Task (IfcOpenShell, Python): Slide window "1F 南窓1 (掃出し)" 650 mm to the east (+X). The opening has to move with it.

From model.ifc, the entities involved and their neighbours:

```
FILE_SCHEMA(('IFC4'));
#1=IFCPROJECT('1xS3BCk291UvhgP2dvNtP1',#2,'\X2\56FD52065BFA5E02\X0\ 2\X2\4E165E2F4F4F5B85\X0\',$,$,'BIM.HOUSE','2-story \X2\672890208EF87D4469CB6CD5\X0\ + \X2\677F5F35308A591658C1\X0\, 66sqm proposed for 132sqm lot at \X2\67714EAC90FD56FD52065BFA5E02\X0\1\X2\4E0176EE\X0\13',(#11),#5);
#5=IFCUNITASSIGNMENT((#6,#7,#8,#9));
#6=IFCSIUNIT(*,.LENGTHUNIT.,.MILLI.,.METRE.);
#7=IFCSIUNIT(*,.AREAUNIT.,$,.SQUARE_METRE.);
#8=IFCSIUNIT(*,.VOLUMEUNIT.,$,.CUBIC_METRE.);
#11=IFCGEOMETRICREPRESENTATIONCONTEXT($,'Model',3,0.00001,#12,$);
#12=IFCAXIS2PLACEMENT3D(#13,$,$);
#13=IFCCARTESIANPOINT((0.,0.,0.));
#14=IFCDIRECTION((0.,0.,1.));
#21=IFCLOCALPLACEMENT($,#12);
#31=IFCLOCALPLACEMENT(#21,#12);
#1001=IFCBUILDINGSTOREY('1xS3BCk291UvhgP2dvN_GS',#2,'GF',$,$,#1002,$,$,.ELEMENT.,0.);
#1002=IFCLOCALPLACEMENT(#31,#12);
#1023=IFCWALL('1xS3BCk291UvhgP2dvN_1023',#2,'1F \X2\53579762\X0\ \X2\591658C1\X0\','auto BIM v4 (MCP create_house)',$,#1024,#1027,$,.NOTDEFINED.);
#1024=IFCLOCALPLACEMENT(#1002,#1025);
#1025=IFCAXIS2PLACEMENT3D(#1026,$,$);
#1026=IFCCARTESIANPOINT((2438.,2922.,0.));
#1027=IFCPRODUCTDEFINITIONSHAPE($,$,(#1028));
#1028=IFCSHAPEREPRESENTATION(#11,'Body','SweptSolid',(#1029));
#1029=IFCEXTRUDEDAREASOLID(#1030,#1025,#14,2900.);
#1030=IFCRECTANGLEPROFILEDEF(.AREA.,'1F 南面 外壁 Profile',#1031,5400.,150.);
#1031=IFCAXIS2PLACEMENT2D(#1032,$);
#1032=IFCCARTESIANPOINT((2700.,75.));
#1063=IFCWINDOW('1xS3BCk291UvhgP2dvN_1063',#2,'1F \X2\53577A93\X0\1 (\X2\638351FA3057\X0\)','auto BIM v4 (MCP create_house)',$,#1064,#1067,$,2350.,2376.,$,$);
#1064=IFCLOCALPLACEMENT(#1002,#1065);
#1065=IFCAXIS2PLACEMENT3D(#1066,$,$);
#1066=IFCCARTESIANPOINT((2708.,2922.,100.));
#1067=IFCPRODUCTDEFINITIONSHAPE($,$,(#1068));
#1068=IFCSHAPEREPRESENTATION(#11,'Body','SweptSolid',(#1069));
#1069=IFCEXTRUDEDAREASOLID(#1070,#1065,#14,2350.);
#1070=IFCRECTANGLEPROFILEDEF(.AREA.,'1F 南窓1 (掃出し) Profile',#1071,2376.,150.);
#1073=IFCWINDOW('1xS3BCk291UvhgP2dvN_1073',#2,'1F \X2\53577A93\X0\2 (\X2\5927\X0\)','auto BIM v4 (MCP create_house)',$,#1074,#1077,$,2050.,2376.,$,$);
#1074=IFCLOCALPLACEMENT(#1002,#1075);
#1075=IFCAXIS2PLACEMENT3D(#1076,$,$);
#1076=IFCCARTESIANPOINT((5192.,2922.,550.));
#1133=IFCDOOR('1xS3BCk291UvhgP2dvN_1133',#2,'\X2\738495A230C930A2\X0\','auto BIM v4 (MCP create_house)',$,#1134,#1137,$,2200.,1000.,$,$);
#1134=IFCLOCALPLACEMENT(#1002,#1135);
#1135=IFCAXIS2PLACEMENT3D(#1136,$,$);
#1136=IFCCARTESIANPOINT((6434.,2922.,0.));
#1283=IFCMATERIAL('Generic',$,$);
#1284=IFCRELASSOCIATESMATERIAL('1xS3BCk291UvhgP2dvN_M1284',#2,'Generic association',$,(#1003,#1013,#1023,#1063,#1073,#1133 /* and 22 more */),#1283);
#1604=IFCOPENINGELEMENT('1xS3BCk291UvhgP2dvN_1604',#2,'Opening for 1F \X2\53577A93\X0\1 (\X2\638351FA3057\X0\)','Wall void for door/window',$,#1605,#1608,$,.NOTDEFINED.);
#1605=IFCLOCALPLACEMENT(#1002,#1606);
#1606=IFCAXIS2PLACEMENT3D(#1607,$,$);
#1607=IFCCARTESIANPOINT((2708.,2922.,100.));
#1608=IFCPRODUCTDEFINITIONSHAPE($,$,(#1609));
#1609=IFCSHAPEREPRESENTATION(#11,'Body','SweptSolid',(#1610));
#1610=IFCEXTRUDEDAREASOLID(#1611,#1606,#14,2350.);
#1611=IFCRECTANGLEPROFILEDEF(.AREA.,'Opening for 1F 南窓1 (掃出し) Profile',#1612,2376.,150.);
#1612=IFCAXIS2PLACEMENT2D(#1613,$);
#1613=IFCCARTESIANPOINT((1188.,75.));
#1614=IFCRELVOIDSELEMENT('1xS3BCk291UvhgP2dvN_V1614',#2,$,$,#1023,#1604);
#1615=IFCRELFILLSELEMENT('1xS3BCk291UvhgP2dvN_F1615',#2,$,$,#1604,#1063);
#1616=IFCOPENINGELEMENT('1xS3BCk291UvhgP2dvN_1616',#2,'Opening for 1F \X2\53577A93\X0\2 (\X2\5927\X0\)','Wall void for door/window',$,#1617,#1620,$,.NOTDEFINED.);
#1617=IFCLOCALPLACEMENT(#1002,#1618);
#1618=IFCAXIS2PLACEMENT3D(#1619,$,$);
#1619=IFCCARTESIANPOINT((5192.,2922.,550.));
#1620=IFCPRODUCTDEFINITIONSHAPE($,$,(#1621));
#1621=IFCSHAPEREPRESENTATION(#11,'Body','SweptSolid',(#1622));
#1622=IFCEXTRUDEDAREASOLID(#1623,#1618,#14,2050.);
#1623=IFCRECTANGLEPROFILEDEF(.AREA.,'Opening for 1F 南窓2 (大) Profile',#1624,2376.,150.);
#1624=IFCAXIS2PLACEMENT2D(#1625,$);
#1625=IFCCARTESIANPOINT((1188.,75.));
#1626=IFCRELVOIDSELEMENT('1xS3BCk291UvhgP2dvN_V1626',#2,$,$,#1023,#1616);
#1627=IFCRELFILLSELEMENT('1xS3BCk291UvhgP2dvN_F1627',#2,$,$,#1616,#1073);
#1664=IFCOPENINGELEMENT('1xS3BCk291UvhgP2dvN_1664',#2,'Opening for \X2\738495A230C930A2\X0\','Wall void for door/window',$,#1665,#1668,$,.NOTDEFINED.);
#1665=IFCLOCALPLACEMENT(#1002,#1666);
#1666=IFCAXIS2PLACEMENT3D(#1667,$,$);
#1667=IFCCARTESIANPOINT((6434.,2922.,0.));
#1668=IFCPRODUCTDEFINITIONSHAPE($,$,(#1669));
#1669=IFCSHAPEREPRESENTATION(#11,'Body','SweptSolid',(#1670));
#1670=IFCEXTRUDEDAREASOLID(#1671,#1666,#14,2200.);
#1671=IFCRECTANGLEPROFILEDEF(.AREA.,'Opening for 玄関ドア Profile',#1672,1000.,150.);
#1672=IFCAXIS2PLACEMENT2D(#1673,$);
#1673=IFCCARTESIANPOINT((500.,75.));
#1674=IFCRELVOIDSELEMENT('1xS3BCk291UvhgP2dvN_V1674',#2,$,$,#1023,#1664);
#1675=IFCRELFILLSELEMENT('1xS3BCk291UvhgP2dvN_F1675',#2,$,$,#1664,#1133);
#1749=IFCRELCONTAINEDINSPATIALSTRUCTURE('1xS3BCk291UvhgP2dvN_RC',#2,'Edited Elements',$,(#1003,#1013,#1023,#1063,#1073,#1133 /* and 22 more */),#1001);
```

```python
import ifcopenshell
import ifcopenshell.api.geometry
import ifcopenshell.util.placement

model = ifcopenshell.open("model.ifc")

window = model.by_guid("1xS3BCk291UvhgP2dvN_1063")
opening = window.FillsVoids[0].RelatingOpeningElement
wall = opening.VoidsElements[0].RelatingBuildingElement

wall_matrix = ifcopenshell.util.placement.get_local_placement(wall.ObjectPlacement)
shift = wall_matrix[:3, 0] * 650.0
before = ifcopenshell.util.placement.get_local_placement(window.ObjectPlacement)[:3, 3].copy()

# The window is not placed relative to its opening, so move both.
for product in (opening, window):
    matrix = ifcopenshell.util.placement.get_local_placement(product.ObjectPlacement)
    matrix[:3, 3] += shift
    ifcopenshell.api.geometry.edit_object_placement(model, product=product, matrix=matrix, is_si=False)

after = ifcopenshell.util.placement.get_local_placement(window.ObjectPlacement)[:3, 3]
print("window moved by", (after - before).round(3) + 0.0)

model.write("model_edited.ifc")
```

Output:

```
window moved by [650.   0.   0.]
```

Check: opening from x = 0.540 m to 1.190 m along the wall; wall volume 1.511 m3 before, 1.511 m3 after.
